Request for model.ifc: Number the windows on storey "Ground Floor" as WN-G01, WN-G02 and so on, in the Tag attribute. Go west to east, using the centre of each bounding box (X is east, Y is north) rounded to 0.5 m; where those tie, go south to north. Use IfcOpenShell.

First a look at what the model holds.

```python
import ifcopenshell
import ifcopenshell.util.element
import ifcopenshell.util.placement

model = ifcopenshell.open("model.ifc")
print(model.schema)
storey = next(s for s in model.by_type("IfcBuildingStorey") if s.Name == "Ground Floor")
windows = [e for e in ifcopenshell.util.element.get_decomposition(storey) if e.is_a("IfcWindow")]
for e in sorted(windows, key=lambda e: e.id()):
    origin = ifcopenshell.util.placement.get_local_placement(e.ObjectPlacement)[:3, 3]
    print(e.id(), e.Tag, e.Name, origin.round(2) + 0.0, sep=" | ")
```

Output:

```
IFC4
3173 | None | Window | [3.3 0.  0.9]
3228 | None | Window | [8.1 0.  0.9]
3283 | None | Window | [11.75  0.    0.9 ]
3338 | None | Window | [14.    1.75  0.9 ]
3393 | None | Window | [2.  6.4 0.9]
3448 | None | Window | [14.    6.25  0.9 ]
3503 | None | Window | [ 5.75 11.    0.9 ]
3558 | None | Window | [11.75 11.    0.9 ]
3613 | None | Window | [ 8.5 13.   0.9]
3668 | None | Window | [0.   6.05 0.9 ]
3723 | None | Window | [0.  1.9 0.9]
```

```python
import ifcopenshell
import ifcopenshell.geom
import ifcopenshell.util.element
import ifcopenshell.util.shape

model = ifcopenshell.open("model.ifc")
settings = ifcopenshell.geom.settings()
settings.set("use-world-coords", True)


def centre(element):
    shape = ifcopenshell.geom.create_shape(settings, element)
    return ifcopenshell.util.shape.get_bbox_centroid(shape.geometry)


storey = next(s for s in model.by_type("IfcBuildingStorey") if s.Name == "Ground Floor")
windows = [e for e in ifcopenshell.util.element.get_decomposition(storey) if e.is_a("IfcWindow")]

# Insertion points can sit at a corner or the storey origin, so sort by the geometry (in metres).
centres = {e: centre(e) for e in windows}
windows.sort(key=lambda e: (round(centres[e][0] / 0.5), centres[e][1]))

for i, e in enumerate(windows, start=1):
    number = f"WN-G{i:02d}"
    e.Tag = number
    print(e.id(), number)

model.write("model_updated.ifc")
```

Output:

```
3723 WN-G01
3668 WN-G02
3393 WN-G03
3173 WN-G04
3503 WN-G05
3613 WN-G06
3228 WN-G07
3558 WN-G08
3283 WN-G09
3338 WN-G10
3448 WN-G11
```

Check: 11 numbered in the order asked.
